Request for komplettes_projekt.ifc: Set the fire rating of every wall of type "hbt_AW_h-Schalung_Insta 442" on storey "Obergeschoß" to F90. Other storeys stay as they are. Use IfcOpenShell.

First a look at what the model holds.

```python
import ifcopenshell
import ifcopenshell.util.element

model = ifcopenshell.open("komplettes_projekt.ifc")
print(model.schema)
storey = next(s for s in model.by_type("IfcBuildingStorey") if s.Name == "Obergeschoß")
walls = [e for e in ifcopenshell.util.element.get_decomposition(storey) if e.is_a("IfcWall")]
seen = {}
for e in walls:
    element_type = ifcopenshell.util.element.get_type(e)
    key = (element_type.Name if element_type != e and element_type else None, ifcopenshell.util.element.get_pset(e, "Pset_WallCommon", "FireRating"))
    seen[key] = seen.get(key, 0) + 1
for (name, value), count in sorted(seen.items(), key=str):
    print(count, "x", name, "|", value)
```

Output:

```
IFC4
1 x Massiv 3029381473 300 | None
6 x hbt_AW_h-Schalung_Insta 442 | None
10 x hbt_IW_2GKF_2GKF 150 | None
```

```python
import ifcopenshell
import ifcopenshell.api.pset
import ifcopenshell.util.element

model = ifcopenshell.open("komplettes_projekt.ifc")

storey = next(s for s in model.by_type("IfcBuildingStorey") if s.Name == "Obergeschoß")
walls = [e for e in ifcopenshell.util.element.get_decomposition(storey) if e.is_a("IfcWall")]

count = 0
for e in walls:
    element_type = ifcopenshell.util.element.get_type(e)
    if element_type in (None, e) or element_type.Name != "hbt_AW_h-Schalung_Insta 442":
        continue
    # add_pset returns the element's existing set when there is one.
    pset = ifcopenshell.api.pset.add_pset(model, product=e, name="Pset_WallCommon")
    ifcopenshell.api.pset.edit_pset(model, pset=pset, properties={"FireRating": "F90"})
    count += 1

print(count, "walls updated")

model.write("komplettes_projekt-out.ifc")
```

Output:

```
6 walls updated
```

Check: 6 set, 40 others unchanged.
